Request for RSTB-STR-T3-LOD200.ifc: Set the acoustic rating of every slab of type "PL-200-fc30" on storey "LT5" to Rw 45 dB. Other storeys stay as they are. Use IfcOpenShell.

First a look at what the model holds.

```python
import ifcopenshell
import ifcopenshell.util.element

model = ifcopenshell.open("RSTB-STR-T3-LOD200.ifc")
print(model.schema)
storey = next(s for s in model.by_type("IfcBuildingStorey") if s.Name == "LT5")
slabs = [e for e in ifcopenshell.util.element.get_decomposition(storey) if e.is_a("IfcSlab")]
seen = {}
for e in slabs:
    element_type = ifcopenshell.util.element.get_type(e)
    key = (element_type.Name if element_type != e and element_type else None, ifcopenshell.util.element.get_pset(e, "Pset_SlabCommon", "AcousticRating"))
    seen[key] = seen.get(key, 0) + 1
for (name, value), count in sorted(seen.items(), key=str):
    print(count, "x", name, "|", value)
```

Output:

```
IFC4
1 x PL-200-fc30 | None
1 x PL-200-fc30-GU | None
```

```python
import ifcopenshell
import ifcopenshell.api.pset
import ifcopenshell.util.element

model = ifcopenshell.open("RSTB-STR-T3-LOD200.ifc")

storey = next(s for s in model.by_type("IfcBuildingStorey") if s.Name == "LT5")
slabs = [e for e in ifcopenshell.util.element.get_decomposition(storey) if e.is_a("IfcSlab")]

count = 0
for e in slabs:
    element_type = ifcopenshell.util.element.get_type(e)
    if element_type in (None, e) or element_type.Name != "PL-200-fc30":
        continue
    # add_pset returns the element's existing set when there is one.
    pset = ifcopenshell.api.pset.add_pset(model, product=e, name="Pset_SlabCommon")
    ifcopenshell.api.pset.edit_pset(model, pset=pset, properties={"AcousticRating": "Rw 45 dB"})
    count += 1

print(count, "slabs updated")

model.write("RSTB-STR-T3-LOD200_rev.ifc")
```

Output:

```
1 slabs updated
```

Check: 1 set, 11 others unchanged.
